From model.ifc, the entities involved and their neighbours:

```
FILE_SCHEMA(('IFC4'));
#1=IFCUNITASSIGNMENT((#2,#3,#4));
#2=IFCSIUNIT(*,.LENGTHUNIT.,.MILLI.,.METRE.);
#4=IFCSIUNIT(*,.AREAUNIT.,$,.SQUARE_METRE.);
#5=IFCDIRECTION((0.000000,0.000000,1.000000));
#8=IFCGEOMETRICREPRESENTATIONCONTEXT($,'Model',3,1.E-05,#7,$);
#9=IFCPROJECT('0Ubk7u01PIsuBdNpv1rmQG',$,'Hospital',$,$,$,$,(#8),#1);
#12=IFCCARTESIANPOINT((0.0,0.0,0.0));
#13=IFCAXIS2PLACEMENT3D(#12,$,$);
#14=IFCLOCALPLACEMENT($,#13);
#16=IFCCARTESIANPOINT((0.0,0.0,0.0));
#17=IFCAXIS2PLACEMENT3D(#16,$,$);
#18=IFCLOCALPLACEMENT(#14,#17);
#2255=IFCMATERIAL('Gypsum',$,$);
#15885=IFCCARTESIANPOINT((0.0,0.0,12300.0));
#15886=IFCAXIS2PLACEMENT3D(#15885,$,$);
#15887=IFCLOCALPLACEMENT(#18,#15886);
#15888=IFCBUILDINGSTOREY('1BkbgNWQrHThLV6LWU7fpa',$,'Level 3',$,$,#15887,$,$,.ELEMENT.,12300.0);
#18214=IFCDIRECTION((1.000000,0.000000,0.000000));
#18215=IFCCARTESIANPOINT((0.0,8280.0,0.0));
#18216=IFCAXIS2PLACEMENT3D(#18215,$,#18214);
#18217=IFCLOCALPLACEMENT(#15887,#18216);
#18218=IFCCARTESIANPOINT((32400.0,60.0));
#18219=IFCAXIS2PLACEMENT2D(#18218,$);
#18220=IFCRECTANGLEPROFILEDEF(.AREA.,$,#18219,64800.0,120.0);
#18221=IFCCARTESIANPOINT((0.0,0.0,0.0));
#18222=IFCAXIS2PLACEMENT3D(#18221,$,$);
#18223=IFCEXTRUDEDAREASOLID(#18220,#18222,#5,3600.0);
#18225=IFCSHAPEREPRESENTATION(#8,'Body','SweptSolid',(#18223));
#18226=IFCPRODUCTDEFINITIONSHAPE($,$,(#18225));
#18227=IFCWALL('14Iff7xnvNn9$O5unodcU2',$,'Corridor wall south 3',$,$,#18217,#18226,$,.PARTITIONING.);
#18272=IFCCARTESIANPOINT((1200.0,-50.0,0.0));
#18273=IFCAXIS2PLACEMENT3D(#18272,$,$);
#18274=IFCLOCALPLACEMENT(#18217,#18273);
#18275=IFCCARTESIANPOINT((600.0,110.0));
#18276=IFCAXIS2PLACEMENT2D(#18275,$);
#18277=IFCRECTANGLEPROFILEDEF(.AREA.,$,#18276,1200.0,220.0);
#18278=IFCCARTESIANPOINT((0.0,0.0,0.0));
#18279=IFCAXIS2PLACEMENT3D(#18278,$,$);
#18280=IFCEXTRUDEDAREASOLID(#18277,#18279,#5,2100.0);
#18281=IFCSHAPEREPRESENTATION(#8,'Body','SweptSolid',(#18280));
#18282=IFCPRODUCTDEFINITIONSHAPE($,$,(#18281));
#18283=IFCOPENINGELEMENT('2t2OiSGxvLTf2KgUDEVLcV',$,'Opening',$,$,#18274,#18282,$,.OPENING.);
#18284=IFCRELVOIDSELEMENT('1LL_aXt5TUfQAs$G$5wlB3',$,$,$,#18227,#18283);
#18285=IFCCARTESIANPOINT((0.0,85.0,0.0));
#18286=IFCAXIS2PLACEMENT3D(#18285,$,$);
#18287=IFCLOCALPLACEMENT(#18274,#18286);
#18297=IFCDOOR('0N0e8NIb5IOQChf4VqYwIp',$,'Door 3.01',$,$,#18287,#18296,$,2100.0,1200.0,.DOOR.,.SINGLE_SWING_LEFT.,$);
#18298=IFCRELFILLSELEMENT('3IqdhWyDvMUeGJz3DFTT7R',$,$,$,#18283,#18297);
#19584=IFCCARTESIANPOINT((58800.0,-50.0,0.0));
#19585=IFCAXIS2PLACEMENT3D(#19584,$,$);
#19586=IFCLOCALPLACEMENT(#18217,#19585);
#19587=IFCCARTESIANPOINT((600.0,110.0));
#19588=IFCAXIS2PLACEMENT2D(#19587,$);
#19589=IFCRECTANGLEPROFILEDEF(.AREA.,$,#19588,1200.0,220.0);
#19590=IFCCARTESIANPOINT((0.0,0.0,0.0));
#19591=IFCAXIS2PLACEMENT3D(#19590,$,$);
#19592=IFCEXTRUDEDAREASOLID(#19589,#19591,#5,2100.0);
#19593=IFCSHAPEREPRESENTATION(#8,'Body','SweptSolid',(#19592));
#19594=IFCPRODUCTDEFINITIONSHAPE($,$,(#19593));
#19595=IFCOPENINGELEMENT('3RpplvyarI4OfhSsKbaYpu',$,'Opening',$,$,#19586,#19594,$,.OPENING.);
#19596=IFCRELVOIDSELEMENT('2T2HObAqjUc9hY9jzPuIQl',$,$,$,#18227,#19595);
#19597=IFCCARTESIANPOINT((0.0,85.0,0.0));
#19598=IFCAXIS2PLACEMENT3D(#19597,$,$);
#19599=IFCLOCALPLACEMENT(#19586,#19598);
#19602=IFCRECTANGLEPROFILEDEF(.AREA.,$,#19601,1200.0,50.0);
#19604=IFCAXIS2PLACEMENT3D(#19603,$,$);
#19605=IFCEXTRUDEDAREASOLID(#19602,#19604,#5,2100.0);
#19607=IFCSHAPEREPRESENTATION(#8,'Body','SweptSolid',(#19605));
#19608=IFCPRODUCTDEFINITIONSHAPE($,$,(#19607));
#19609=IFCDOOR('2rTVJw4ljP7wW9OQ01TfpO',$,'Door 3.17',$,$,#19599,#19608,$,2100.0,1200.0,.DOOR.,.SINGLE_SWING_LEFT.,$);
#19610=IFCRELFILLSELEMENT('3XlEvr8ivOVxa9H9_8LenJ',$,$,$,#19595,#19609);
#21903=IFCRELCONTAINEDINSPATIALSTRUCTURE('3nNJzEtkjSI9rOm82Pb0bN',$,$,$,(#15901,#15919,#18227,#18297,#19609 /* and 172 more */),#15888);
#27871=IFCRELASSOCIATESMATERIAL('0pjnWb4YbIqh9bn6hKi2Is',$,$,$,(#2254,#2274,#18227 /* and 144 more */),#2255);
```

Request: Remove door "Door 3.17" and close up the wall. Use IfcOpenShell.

```python
import ifcopenshell
import ifcopenshell.api.feature
import ifcopenshell.api.root
import ifcopenshell.geom
import ifcopenshell.util.shape

model = ifcopenshell.open("model.ifc")
settings = ifcopenshell.geom.settings()


def volume(element):
    """Net volume in cubic metres, openings subtracted."""
    shape = ifcopenshell.geom.create_shape(settings, element)
    return ifcopenshell.util.shape.get_volume(shape.geometry)


door = model.by_guid("2rTVJw4ljP7wW9OQ01TfpO")
opening = door.FillsVoids[0].RelatingOpeningElement
wall = opening.VoidsElements[0].RelatingBuildingElement
before = volume(wall)

ifcopenshell.api.root.remove_product(model, product=door)
ifcopenshell.api.feature.remove_feature(model, feature=opening)

after = volume(wall)

print(f"wall volume {before:.3f} -> {after:.3f} m3")

model.write("model-out.ifc")
```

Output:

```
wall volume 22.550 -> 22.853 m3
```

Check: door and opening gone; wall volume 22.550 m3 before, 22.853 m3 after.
